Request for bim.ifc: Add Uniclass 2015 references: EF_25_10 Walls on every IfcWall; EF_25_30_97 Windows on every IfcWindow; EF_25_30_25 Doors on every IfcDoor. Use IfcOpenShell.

First a look at what the model holds.

```python
import ifcopenshell

model = ifcopenshell.open("bim.ifc")
print(model.schema)
print("classifications:", [c.Name for c in model.by_type("IfcClassification")])
for ifc_class in ("IfcDoor", "IfcRoof", "IfcStair", "IfcWall", "IfcWindow"):
    print(ifc_class, len(model.by_type(ifc_class)))
```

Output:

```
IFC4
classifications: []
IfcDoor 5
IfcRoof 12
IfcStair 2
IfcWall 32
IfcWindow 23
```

```python
import ifcopenshell
import ifcopenshell.api.classification

model = ifcopenshell.open("bim.ifc")

system = ifcopenshell.api.classification.add_classification(model, classification="Uniclass 2015")

codes = {
    "IfcWall": ("EF_25_10", "Walls"),
    "IfcWindow": ("EF_25_30_97", "Windows"),
    "IfcDoor": ("EF_25_30_25", "Doors"),
}
for ifc_class, (code, name) in codes.items():
    products = model.by_type(ifc_class)
    ifcopenshell.api.classification.add_reference(
        model, products=products, classification=system, identification=code, name=name
    )
    print(code, len(products))

model.write("bim_v2.ifc")
```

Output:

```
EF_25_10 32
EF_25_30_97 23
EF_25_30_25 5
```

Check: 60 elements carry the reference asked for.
